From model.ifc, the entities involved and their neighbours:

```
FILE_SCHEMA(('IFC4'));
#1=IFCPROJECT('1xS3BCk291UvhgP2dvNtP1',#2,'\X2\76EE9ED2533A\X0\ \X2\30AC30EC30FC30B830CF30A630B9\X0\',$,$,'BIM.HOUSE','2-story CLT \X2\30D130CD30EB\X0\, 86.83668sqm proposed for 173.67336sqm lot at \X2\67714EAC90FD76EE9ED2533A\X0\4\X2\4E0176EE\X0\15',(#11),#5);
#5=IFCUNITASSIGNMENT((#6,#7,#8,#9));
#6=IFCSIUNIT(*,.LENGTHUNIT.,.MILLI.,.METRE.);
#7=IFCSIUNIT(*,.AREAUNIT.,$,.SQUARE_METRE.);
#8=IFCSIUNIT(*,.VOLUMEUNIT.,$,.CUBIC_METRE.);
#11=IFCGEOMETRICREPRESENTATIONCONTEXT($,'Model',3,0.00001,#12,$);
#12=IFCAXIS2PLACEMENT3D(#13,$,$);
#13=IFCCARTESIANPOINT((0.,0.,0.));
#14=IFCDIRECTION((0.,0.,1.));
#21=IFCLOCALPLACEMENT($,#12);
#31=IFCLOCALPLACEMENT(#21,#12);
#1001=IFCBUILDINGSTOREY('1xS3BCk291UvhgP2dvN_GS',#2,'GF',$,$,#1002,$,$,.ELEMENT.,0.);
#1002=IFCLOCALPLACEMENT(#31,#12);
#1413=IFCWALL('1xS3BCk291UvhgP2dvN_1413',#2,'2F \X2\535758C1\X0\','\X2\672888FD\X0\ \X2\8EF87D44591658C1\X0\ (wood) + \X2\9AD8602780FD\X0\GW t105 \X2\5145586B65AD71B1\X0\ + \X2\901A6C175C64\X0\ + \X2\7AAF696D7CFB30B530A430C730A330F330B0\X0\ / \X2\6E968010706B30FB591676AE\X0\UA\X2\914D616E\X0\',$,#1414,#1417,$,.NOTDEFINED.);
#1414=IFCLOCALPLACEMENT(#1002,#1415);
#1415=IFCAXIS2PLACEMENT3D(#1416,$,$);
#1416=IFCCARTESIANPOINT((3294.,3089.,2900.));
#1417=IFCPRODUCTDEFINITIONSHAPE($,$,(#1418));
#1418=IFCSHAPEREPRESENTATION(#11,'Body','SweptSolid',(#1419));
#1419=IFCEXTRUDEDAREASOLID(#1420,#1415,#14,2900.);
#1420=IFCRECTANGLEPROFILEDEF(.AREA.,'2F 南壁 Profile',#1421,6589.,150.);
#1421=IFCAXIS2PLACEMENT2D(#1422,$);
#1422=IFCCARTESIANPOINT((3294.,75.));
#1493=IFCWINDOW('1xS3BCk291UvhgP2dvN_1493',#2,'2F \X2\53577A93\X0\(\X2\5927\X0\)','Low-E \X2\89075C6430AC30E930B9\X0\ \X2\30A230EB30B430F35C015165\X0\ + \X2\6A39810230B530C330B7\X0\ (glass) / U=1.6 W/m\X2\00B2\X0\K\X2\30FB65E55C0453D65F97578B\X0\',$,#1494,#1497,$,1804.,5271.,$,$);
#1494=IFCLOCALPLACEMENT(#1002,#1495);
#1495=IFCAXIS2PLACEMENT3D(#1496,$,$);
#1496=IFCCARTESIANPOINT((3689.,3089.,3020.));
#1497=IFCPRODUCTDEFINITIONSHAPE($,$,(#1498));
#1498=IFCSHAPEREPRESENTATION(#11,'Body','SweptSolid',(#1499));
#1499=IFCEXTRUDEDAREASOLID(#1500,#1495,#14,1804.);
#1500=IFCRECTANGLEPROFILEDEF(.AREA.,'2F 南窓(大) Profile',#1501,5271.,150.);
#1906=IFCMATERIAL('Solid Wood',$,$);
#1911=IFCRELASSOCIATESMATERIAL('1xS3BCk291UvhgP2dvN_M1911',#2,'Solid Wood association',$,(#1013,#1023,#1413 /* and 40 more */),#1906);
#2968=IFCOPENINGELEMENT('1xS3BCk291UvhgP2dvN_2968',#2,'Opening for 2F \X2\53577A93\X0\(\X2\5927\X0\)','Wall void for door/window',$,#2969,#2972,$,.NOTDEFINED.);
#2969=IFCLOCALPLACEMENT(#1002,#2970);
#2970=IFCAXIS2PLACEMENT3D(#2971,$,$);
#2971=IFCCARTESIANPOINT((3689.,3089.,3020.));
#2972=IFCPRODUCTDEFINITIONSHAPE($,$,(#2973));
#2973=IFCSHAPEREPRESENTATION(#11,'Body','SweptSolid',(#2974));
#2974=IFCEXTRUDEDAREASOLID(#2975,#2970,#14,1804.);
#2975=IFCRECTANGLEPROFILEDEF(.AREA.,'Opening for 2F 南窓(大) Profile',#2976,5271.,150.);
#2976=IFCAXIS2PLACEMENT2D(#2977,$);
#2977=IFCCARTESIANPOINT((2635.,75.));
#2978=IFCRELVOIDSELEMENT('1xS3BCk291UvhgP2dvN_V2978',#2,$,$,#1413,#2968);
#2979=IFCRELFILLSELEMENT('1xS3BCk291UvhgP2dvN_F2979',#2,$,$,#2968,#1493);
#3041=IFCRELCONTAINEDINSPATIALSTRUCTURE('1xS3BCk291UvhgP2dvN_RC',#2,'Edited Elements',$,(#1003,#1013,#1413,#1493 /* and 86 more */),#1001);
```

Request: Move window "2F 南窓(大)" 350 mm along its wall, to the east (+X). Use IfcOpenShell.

```python
import ifcopenshell
import ifcopenshell.api.geometry
import ifcopenshell.util.placement
import ifcopenshell.util.unit

model = ifcopenshell.open("model.ifc")
unit_scale = ifcopenshell.util.unit.calculate_unit_scale(model)

window = model.by_guid("1xS3BCk291UvhgP2dvN_1493")
opening = window.FillsVoids[0].RelatingOpeningElement
wall = opening.VoidsElements[0].RelatingBuildingElement

wall_matrix = ifcopenshell.util.placement.get_local_placement(wall.ObjectPlacement)
shift = wall_matrix[:3, 0] * 0.35 / unit_scale
before = ifcopenshell.util.placement.get_local_placement(window.ObjectPlacement)[:3, 3].copy()

# The window is not placed relative to its opening, so move both.
for product in (opening, window):
    matrix = ifcopenshell.util.placement.get_local_placement(product.ObjectPlacement)
    matrix[:3, 3] += shift
    ifcopenshell.api.geometry.edit_object_placement(model, product=product, matrix=matrix, is_si=False)

after = ifcopenshell.util.placement.get_local_placement(window.ObjectPlacement)[:3, 3]
print("window moved by", (after - before).round(3) + 0.0)

model.write("model_rev.ifc")
```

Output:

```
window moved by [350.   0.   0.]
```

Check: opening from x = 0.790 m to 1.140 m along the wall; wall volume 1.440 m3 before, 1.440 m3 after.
